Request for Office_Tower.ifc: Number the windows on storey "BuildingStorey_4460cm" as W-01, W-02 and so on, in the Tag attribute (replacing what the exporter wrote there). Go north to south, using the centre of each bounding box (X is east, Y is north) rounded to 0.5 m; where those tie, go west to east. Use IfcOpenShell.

First a look at what the model holds.

```python
import ifcopenshell
import ifcopenshell.util.element
import ifcopenshell.util.placement

model = ifcopenshell.open("Office_Tower.ifc")
print(model.schema)
storey = next(s for s in model.by_type("IfcBuildingStorey") if s.Name == "BuildingStorey_4460cm")
windows = [e for e in ifcopenshell.util.element.get_decomposition(storey) if e.is_a("IfcWindow")]
for e in sorted(windows, key=lambda e: e.id()):
    origin = ifcopenshell.util.placement.get_local_placement(e.ObjectPlacement)[:3, 3]
    print(e.id(), e.Tag, e.Name, origin.round(2) + 0.0, sep=" | ")
```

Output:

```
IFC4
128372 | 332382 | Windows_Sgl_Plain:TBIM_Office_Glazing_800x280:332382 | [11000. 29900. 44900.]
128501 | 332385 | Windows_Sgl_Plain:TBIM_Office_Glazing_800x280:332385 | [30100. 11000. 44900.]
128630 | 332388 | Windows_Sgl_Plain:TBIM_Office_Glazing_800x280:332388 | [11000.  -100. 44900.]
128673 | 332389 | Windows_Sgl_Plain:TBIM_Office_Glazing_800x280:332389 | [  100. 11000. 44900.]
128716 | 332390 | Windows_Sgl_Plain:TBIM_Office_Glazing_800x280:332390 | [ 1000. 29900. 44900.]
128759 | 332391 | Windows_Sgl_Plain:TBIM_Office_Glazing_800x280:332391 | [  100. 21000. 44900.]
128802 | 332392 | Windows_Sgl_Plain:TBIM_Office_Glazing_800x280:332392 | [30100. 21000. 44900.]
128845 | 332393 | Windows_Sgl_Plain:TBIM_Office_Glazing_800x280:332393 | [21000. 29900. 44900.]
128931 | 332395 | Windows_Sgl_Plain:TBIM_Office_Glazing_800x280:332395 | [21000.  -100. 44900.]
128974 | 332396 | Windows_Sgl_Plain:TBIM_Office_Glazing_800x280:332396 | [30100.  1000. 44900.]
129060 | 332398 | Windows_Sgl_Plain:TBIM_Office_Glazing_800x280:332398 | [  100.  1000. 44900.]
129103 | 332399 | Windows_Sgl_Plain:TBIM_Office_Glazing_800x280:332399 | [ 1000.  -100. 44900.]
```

```python
import ifcopenshell
import ifcopenshell.geom
import ifcopenshell.util.element
import ifcopenshell.util.shape

model = ifcopenshell.open("Office_Tower.ifc")
settings = ifcopenshell.geom.settings()
settings.set("use-world-coords", True)


def centre(element):
    shape = ifcopenshell.geom.create_shape(settings, element)
    return ifcopenshell.util.shape.get_bbox_centroid(shape.geometry)


storey = next(s for s in model.by_type("IfcBuildingStorey") if s.Name == "BuildingStorey_4460cm")
windows = [e for e in ifcopenshell.util.element.get_decomposition(storey) if e.is_a("IfcWindow")]

# Insertion points can sit at a corner or the storey origin, so sort by the geometry (in metres).
centres = {e: centre(e) for e in windows}
windows.sort(key=lambda e: (-round(centres[e][1] / 0.5), centres[e][0]))

for i, e in enumerate(windows, start=1):
    number = f"W-{i:02d}"
    e.Tag = number
    print(e.id(), number)

model.write("Office_Tower_edited.ifc")
```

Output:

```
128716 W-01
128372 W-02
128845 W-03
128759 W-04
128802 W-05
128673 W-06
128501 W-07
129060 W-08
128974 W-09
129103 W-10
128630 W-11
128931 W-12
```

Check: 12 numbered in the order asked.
